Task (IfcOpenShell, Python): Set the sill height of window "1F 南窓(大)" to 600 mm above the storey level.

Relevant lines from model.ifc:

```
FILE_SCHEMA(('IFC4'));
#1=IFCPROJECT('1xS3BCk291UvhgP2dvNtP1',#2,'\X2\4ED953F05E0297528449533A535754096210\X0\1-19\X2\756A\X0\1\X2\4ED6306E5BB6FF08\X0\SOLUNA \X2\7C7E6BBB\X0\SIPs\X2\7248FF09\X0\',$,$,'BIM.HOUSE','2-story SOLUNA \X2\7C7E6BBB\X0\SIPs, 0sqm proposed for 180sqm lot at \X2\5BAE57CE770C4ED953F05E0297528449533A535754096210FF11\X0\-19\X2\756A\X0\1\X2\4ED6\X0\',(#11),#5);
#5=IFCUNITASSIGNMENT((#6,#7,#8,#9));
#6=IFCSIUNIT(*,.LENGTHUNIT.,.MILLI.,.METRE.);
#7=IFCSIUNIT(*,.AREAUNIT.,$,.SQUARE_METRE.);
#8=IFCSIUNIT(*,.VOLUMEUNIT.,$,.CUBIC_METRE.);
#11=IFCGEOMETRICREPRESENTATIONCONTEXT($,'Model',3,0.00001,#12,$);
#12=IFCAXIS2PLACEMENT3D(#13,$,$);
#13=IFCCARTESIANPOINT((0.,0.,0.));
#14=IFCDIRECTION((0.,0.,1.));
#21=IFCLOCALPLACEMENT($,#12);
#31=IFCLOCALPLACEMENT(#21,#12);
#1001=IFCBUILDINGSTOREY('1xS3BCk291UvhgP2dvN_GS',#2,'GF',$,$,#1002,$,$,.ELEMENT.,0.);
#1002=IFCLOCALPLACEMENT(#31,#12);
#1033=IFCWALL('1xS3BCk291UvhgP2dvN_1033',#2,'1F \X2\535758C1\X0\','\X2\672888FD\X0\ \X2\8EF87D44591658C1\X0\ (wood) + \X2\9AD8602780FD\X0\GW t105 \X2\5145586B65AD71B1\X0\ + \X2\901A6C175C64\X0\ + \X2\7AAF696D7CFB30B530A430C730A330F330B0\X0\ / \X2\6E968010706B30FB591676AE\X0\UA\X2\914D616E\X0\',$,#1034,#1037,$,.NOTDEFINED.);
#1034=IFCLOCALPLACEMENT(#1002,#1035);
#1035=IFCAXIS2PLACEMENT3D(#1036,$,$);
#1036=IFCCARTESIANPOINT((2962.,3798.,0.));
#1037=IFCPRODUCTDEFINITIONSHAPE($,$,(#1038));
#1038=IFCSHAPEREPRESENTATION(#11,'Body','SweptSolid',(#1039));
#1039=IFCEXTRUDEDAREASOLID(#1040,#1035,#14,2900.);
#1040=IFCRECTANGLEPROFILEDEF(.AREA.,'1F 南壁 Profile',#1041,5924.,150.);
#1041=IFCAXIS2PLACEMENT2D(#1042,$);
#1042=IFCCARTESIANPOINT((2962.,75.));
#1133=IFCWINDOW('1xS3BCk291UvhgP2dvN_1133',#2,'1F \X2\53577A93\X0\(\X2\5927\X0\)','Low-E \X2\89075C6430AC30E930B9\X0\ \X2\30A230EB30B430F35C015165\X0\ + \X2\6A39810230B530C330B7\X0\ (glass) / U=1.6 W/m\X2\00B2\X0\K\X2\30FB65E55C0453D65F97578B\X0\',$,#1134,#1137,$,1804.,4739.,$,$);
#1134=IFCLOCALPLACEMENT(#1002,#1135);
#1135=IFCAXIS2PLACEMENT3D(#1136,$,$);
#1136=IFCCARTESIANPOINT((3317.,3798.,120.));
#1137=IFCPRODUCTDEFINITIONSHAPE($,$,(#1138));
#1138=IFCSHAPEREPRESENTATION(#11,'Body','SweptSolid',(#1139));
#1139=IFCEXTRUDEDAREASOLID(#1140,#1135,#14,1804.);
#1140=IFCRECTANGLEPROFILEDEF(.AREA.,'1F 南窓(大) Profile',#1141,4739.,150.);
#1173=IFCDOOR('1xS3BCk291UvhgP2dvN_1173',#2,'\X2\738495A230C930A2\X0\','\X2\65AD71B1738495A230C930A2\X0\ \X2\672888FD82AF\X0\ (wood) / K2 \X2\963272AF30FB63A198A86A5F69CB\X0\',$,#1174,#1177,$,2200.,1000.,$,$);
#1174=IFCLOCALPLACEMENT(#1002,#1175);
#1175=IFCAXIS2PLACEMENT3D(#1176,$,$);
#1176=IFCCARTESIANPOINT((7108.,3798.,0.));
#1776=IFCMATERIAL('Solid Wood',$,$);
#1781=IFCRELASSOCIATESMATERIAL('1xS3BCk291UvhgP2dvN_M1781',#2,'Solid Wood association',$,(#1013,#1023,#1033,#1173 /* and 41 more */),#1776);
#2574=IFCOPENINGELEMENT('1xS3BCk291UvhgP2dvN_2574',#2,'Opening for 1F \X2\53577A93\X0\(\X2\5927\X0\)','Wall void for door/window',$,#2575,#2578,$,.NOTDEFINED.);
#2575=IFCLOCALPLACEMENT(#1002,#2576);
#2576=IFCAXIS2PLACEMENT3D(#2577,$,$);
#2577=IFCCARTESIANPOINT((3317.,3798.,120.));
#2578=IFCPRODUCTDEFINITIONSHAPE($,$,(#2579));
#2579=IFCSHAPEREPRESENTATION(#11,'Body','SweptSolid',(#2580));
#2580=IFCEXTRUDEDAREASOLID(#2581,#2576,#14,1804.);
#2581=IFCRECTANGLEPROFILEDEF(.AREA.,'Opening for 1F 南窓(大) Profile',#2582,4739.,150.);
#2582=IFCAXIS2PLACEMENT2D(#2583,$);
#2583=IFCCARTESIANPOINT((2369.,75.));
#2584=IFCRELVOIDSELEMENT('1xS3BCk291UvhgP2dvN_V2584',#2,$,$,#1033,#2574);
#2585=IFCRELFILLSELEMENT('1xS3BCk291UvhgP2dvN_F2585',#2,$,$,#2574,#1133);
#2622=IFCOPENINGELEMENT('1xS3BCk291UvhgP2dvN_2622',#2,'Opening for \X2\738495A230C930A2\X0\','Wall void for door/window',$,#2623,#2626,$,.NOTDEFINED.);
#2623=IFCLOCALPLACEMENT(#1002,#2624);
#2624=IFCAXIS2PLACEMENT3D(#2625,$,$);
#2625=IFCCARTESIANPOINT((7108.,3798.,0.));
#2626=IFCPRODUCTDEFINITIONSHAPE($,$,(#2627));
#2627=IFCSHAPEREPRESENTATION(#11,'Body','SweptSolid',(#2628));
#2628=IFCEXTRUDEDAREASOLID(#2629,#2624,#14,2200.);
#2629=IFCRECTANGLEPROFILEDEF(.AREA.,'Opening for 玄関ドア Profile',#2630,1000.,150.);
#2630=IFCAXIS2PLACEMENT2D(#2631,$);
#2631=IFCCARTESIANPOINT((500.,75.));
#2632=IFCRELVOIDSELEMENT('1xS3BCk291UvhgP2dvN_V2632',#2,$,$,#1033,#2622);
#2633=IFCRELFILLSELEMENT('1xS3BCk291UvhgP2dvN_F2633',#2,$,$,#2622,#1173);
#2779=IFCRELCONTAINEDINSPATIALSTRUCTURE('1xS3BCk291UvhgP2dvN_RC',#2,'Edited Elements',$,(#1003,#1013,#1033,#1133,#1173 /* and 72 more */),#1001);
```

```python
import numpy as np
import ifcopenshell
import ifcopenshell.api.geometry
import ifcopenshell.geom
import ifcopenshell.util.element
import ifcopenshell.util.placement
import ifcopenshell.util.shape
import ifcopenshell.util.unit

model = ifcopenshell.open("model.ifc")
unit_scale = ifcopenshell.util.unit.calculate_unit_scale(model)

window = model.by_guid("1xS3BCk291UvhgP2dvN_1133")
opening = window.FillsVoids[0].RelatingOpeningElement
storey = ifcopenshell.util.element.get_container(window, ifc_class="IfcBuildingStorey")
level = ifcopenshell.util.placement.get_local_placement(storey.ObjectPlacement)[2, 3]

# The opening's origin need not be at the sill, so measure its lowest point.
shape = ifcopenshell.geom.create_shape(ifcopenshell.geom.settings(), opening)
bottom = ifcopenshell.util.shape.get_shape_bottom_elevation(shape, shape.geometry) / unit_scale
dz = level + 0.6 / unit_scale - bottom

shift = np.array([0.0, 0.0, dz])
# The window is not placed relative to its opening, so move both.
for product in (opening, window):
    matrix = ifcopenshell.util.placement.get_local_placement(product.ObjectPlacement)
    matrix[:3, 3] += shift
    ifcopenshell.api.geometry.edit_object_placement(model, product=product, matrix=matrix, is_si=False)

print(f"moved by {dz * unit_scale:+.3f} m")

model.write("model_updated.ifc")
```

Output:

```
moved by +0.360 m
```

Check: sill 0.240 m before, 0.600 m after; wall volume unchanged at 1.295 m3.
